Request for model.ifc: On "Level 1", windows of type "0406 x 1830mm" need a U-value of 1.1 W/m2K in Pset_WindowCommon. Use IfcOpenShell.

First a look at what the model holds.

```python
import ifcopenshell
import ifcopenshell.util.element

model = ifcopenshell.open("model.ifc")
print(model.schema)
storey = next(s for s in model.by_type("IfcBuildingStorey") if s.Name == "Level 1")
windows = [e for e in ifcopenshell.util.element.get_decomposition(storey) if e.is_a("IfcWindow")]
seen = {}
for e in windows:
    element_type = ifcopenshell.util.element.get_type(e)
    key = (element_type.Name if element_type != e and element_type else None, ifcopenshell.util.element.get_pset(e, "Pset_WindowCommon", "ThermalTransmittance"))
    seen[key] = seen.get(key, 0) + 1
for (name, value), count in sorted(seen.items(), key=str):
    print(count, "x", name, "|", value)
```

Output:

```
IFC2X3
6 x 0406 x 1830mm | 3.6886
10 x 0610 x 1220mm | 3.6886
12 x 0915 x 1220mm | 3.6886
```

```python
import ifcopenshell
import ifcopenshell.api.pset
import ifcopenshell.util.element

model = ifcopenshell.open("model.ifc")

storey = next(s for s in model.by_type("IfcBuildingStorey") if s.Name == "Level 1")
windows = [e for e in ifcopenshell.util.element.get_decomposition(storey) if e.is_a("IfcWindow")]

count = 0
for e in windows:
    element_type = ifcopenshell.util.element.get_type(e)
    if element_type in (None, e) or element_type.Name != "0406 x 1830mm":
        continue
    # add_pset returns the element's existing set when there is one.
    pset = ifcopenshell.api.pset.add_pset(model, product=e, name="Pset_WindowCommon")
    ifcopenshell.api.pset.edit_pset(model, pset=pset, properties={"ThermalTransmittance": 1.1})
    count += 1

print(count, "windows updated")

model.write("model_rev.ifc")
```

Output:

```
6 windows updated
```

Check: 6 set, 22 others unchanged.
